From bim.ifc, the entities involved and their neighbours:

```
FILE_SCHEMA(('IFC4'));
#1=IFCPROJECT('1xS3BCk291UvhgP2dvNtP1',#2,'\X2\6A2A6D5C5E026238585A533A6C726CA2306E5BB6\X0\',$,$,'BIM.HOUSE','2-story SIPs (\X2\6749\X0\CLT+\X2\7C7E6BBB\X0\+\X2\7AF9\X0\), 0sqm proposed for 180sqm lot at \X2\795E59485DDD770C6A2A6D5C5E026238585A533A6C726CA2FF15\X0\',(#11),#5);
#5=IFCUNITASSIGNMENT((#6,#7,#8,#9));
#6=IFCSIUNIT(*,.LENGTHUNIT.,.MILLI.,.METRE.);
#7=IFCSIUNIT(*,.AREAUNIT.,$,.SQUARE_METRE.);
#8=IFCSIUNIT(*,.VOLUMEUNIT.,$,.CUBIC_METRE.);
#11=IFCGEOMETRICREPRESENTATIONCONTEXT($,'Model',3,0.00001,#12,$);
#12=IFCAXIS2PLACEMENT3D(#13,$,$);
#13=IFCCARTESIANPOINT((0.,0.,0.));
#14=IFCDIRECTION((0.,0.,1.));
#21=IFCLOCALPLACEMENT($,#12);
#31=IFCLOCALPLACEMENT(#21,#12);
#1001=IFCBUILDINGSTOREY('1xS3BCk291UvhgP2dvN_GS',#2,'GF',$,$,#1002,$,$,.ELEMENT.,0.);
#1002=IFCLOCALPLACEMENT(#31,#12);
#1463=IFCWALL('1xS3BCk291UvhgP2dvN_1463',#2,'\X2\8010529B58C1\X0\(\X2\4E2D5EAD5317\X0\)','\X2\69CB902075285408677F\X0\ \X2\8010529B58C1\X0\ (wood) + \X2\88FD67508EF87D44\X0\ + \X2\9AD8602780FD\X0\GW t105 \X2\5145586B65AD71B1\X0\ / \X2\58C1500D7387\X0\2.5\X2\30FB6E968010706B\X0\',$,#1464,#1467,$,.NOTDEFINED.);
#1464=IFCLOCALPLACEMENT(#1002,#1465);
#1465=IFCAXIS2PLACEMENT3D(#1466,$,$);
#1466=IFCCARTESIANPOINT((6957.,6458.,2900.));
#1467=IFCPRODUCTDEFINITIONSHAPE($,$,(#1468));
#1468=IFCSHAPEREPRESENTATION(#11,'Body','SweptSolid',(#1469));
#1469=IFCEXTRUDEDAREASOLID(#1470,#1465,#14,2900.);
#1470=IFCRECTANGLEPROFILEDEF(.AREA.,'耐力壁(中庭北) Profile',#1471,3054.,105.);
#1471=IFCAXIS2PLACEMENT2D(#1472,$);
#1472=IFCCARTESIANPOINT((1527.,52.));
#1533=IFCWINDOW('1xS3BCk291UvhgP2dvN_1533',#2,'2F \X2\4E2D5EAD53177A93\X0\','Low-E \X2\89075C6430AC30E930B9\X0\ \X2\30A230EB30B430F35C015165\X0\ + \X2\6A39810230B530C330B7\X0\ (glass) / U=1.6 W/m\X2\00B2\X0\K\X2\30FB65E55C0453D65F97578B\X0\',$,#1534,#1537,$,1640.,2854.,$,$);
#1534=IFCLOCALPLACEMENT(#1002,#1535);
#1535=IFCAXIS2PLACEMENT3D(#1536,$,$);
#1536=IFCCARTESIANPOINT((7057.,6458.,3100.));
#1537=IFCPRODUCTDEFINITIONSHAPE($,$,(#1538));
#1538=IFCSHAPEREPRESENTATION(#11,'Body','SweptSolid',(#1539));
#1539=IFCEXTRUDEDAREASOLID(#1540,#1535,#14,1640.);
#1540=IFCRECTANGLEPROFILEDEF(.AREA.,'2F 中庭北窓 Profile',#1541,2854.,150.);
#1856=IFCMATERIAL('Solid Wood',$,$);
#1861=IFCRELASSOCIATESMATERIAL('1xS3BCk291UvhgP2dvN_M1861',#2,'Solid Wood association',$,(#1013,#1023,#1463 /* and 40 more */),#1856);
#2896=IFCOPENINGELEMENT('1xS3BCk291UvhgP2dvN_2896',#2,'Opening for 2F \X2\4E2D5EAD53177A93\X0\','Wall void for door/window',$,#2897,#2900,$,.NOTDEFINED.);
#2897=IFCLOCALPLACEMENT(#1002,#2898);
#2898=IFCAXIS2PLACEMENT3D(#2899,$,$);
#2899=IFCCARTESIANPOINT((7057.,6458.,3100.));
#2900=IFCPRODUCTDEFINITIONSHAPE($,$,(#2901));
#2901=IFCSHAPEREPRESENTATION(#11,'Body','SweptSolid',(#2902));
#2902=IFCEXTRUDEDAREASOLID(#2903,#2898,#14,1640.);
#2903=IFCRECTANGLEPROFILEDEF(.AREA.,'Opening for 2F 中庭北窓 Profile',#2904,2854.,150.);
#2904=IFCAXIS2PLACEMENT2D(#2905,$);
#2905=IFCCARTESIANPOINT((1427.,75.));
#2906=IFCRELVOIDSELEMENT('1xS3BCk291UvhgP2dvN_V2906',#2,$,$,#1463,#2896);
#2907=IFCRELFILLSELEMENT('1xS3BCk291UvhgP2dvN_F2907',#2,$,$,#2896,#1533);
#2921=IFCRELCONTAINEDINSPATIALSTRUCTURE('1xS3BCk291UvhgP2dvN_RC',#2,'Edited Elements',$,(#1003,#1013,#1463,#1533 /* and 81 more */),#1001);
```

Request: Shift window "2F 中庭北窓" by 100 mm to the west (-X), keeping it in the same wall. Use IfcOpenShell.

```python
import ifcopenshell
import ifcopenshell.api.geometry
import ifcopenshell.util.placement
import ifcopenshell.util.unit

model = ifcopenshell.open("bim.ifc")
unit_scale = ifcopenshell.util.unit.calculate_unit_scale(model)

window = model.by_guid("1xS3BCk291UvhgP2dvN_1533")
opening = window.FillsVoids[0].RelatingOpeningElement
wall = opening.VoidsElements[0].RelatingBuildingElement

wall_matrix = ifcopenshell.util.placement.get_local_placement(wall.ObjectPlacement)
shift = wall_matrix[:3, 0] * -0.1 / unit_scale
before = ifcopenshell.util.placement.get_local_placement(window.ObjectPlacement)[:3, 3].copy()

# The window is not placed relative to its opening, so move both.
for product in (opening, window):
    matrix = ifcopenshell.util.placement.get_local_placement(product.ObjectPlacement)
    matrix[:3, 3] += shift
    ifcopenshell.api.geometry.edit_object_placement(model, product=product, matrix=matrix, is_si=False)

after = ifcopenshell.util.placement.get_local_placement(window.ObjectPlacement)[:3, 3]
print("window moved by", (after - before).round(3) + 0.0)

model.write("bim_updated.ifc")
```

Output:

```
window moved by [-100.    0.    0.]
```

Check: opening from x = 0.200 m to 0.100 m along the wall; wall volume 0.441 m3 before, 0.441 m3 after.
